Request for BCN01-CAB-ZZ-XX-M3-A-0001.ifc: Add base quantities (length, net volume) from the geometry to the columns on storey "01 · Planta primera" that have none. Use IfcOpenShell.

First a look at what the model holds.

```python
import ifcopenshell
import ifcopenshell.util.element
import ifcopenshell.util.unit

model = ifcopenshell.open("BCN01-CAB-ZZ-XX-M3-A-0001.ifc")
print(model.schema)
for unit_type in ("LENGTHUNIT", "AREAUNIT", "VOLUMEUNIT"):
    print(unit_type, ifcopenshell.util.unit.calculate_unit_scale(model, unit_type))
storey = next(s for s in model.by_type("IfcBuildingStorey") if s.Name == "01 · Planta primera")
columns = [e for e in ifcopenshell.util.element.get_decomposition(storey) if e.is_a("IfcColumn")]
for e in sorted(columns, key=lambda e: e.id()):
    print(e.id(), e.is_a(), e.Name, list(ifcopenshell.util.element.get_psets(e, qtos_only=True)), sep=" | ")
```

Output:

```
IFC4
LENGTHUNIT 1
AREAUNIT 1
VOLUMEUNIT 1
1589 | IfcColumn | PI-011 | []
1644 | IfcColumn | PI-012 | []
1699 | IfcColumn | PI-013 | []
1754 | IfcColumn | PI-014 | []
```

```python
import ifcopenshell
import ifcopenshell.api.pset
import ifcopenshell.geom
import ifcopenshell.util.element
import ifcopenshell.util.shape
import ifcopenshell.util.unit

model = ifcopenshell.open("BCN01-CAB-ZZ-XX-M3-A-0001.ifc")
unit_scale = ifcopenshell.util.unit.calculate_unit_scale(model)
volume_scale = ifcopenshell.util.unit.calculate_unit_scale(model, "VOLUMEUNIT")
settings = ifcopenshell.geom.settings()

storey = next(s for s in model.by_type("IfcBuildingStorey") if s.Name == "01 · Planta primera")
columns = [e for e in ifcopenshell.util.element.get_decomposition(storey) if e.is_a("IfcColumn")]

for e in sorted(columns, key=lambda e: e.id()):
    if ifcopenshell.util.element.get_psets(e, qtos_only=True, should_inherit=False):
        continue
    # Geometry comes back in metres, in the element's own axes.
    shape = ifcopenshell.geom.create_shape(settings, e)
    values = {
        "Length": ifcopenshell.util.shape.get_z(shape.geometry) / unit_scale,
        "NetVolume": ifcopenshell.util.shape.get_volume(shape.geometry) / volume_scale,
    }
    qto = ifcopenshell.api.pset.add_qto(model, product=e, name="Qto_ColumnBaseQuantities")
    ifcopenshell.api.pset.edit_qto(model, qto=qto, properties=values)
    print(e.id(), {k: round(v, 3) for k, v in values.items()})

model.write("BCN01-CAB-ZZ-XX-M3-A-0001-out.ifc")
```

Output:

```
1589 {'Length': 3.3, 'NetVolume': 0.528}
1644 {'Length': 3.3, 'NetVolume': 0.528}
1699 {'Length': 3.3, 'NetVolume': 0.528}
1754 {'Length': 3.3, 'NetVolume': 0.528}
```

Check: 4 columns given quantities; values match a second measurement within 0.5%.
